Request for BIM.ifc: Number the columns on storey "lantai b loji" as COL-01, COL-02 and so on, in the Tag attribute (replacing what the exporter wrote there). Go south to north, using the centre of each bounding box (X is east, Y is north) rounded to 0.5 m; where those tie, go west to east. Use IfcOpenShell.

First a look at what the model holds.

```python
import ifcopenshell
import ifcopenshell.util.element
import ifcopenshell.util.placement

model = ifcopenshell.open("BIM.ifc")
print(model.schema)
storey = next(s for s in model.by_type("IfcBuildingStorey") if s.Name == "lantai b loji")
columns = [e for e in ifcopenshell.util.element.get_decomposition(storey) if e.is_a("IfcColumn")]
for e in sorted(columns, key=lambda e: e.id()):
    origin = ifcopenshell.util.placement.get_local_placement(e.ObjectPlacement)[:3, 3]
    print(e.id(), e.Tag, e.Name, origin.round(2) + 0.0, sep=" | ")
```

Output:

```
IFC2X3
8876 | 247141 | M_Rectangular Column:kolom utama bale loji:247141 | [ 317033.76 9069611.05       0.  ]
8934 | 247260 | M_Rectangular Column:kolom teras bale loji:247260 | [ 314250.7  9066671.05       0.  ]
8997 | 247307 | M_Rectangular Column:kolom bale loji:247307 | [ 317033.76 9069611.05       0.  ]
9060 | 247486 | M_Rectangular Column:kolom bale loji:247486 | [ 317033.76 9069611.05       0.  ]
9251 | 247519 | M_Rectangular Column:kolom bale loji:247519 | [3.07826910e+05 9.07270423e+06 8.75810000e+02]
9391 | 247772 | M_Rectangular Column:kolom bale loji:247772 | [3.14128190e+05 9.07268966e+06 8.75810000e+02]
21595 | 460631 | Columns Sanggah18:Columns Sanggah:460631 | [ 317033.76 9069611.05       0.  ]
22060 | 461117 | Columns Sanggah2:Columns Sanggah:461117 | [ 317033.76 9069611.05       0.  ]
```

```python
import ifcopenshell
import ifcopenshell.geom
import ifcopenshell.util.element
import ifcopenshell.util.shape

model = ifcopenshell.open("BIM.ifc")
settings = ifcopenshell.geom.settings()
settings.set("use-world-coords", True)


def centre(element):
    shape = ifcopenshell.geom.create_shape(settings, element)
    return ifcopenshell.util.shape.get_bbox_centroid(shape.geometry)


storey = next(s for s in model.by_type("IfcBuildingStorey") if s.Name == "lantai b loji")
columns = [e for e in ifcopenshell.util.element.get_decomposition(storey) if e.is_a("IfcColumn")]

# Insertion points can sit at a corner or the storey origin, so sort by the geometry (in metres).
centres = {e: centre(e) for e in columns}
columns.sort(key=lambda e: (round(centres[e][1] / 0.5), centres[e][0]))

for i, e in enumerate(columns, start=1):
    number = f"COL-{i:02d}"
    e.Tag = number
    print(e.id(), number)

model.write("BIM_edited.ifc")
```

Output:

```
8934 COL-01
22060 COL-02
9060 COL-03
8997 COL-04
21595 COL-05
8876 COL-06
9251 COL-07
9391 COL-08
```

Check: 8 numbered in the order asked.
